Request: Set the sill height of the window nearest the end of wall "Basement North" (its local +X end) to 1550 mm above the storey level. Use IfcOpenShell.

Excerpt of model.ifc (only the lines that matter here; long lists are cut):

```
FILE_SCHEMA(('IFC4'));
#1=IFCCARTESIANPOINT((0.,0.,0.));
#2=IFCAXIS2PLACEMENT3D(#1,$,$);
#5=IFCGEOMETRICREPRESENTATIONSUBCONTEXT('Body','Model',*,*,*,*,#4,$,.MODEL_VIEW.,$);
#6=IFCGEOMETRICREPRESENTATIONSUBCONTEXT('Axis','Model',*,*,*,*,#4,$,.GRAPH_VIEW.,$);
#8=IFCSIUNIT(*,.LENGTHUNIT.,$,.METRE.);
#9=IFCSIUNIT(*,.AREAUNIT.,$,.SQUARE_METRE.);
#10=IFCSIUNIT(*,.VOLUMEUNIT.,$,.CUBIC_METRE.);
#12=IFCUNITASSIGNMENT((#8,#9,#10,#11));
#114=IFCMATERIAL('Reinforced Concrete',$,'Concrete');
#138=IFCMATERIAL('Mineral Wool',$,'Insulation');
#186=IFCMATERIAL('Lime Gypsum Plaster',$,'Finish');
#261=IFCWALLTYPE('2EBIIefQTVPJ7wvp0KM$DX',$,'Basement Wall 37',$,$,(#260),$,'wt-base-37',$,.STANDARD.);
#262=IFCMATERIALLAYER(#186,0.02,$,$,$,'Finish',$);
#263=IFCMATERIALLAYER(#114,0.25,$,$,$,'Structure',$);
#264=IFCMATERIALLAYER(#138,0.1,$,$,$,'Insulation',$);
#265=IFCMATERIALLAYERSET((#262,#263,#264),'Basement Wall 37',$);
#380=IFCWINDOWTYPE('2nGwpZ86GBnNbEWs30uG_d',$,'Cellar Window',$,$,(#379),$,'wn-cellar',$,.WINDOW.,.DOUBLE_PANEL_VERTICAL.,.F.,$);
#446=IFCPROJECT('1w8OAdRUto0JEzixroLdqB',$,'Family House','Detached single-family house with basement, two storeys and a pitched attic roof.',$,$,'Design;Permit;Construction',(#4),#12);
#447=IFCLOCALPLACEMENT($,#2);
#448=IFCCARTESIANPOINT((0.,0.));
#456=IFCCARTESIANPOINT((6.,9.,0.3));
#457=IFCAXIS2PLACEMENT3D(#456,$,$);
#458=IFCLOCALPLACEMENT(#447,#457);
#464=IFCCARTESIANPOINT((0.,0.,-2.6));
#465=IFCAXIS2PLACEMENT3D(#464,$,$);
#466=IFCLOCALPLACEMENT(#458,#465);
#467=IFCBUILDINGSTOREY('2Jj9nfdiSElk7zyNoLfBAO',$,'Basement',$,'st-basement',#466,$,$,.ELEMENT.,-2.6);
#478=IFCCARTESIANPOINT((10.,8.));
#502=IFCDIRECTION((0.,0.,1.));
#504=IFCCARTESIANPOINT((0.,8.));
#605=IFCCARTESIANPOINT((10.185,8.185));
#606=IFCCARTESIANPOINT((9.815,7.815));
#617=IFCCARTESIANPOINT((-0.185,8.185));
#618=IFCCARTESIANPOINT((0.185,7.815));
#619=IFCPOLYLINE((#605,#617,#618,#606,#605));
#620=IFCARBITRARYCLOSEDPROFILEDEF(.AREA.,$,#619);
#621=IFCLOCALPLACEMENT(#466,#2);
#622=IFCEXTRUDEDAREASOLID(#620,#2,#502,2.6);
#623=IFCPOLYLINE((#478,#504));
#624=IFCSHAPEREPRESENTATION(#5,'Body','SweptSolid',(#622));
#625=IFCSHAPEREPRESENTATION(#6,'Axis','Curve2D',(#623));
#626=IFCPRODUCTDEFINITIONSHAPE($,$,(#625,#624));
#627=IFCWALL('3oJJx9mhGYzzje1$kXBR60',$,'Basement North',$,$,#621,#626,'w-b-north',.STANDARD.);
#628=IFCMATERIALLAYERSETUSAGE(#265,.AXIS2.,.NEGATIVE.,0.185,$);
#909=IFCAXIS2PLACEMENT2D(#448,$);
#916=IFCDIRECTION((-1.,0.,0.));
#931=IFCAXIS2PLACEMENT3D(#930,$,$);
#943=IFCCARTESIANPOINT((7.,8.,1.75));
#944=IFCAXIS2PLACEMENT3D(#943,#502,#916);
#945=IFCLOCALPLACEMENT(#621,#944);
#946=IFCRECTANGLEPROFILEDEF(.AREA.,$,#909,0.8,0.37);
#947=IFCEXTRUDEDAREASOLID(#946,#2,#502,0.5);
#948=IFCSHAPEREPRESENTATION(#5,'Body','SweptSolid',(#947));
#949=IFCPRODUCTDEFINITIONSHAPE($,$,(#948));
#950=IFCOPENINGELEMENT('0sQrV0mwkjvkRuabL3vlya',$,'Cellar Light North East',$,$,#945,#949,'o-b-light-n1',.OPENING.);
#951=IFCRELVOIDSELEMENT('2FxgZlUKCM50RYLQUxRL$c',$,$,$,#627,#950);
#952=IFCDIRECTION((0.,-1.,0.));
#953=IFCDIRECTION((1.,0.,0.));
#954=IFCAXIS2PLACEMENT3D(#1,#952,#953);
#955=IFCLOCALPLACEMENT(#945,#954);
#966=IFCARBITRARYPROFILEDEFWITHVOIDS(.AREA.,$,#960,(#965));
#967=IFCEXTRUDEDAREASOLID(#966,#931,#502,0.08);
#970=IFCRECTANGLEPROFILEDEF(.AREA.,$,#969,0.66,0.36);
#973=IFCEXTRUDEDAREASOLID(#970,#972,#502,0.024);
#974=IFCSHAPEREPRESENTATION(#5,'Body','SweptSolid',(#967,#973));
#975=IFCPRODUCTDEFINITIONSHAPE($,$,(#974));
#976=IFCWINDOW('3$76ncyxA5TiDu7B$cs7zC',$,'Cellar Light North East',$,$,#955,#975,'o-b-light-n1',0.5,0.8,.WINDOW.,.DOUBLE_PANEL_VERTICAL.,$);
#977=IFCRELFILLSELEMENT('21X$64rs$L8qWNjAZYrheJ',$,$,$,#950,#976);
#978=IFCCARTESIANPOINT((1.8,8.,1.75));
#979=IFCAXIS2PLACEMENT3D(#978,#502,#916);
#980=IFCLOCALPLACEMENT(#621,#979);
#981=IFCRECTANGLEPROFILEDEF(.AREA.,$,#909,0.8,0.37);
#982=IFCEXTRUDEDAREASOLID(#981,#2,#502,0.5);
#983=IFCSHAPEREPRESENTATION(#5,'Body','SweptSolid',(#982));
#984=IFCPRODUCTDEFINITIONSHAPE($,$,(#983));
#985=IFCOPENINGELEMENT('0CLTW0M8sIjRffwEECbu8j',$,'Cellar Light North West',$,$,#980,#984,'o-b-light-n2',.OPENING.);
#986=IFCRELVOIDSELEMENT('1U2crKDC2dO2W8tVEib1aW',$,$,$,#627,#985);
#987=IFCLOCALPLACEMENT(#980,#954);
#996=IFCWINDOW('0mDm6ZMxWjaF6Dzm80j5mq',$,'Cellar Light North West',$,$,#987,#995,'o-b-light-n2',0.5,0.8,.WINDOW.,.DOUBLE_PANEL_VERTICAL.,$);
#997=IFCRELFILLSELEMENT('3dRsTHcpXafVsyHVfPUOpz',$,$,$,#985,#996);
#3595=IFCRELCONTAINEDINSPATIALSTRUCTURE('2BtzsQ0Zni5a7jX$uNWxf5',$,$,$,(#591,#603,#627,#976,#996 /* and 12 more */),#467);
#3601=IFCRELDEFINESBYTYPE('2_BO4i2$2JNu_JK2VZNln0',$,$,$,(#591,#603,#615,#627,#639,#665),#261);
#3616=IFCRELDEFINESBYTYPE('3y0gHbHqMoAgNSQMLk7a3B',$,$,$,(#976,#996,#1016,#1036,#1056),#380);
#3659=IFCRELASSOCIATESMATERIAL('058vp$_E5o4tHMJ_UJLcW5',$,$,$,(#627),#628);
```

```python
import numpy as np
import ifcopenshell
import ifcopenshell.api.geometry
import ifcopenshell.geom
import ifcopenshell.util.element
import ifcopenshell.util.placement
import ifcopenshell.util.shape
import ifcopenshell.util.unit

model = ifcopenshell.open("model.ifc")
unit_scale = ifcopenshell.util.unit.calculate_unit_scale(model)

window = model.by_guid("3$76ncyxA5TiDu7B$cs7zC")
opening = window.FillsVoids[0].RelatingOpeningElement
storey = ifcopenshell.util.element.get_container(window, ifc_class="IfcBuildingStorey")
level = ifcopenshell.util.placement.get_local_placement(storey.ObjectPlacement)[2, 3]

# The opening's origin need not be at the sill, so measure its lowest point.
shape = ifcopenshell.geom.create_shape(ifcopenshell.geom.settings(), opening)
bottom = ifcopenshell.util.shape.get_shape_bottom_elevation(shape, shape.geometry) / unit_scale
dz = level + 1.55 - bottom

shift = np.array([0.0, 0.0, dz])
# The window is placed relative to its opening, so it follows when the opening moves.
matrix = ifcopenshell.util.placement.get_local_placement(opening.ObjectPlacement)
matrix[:3, 3] += shift
ifcopenshell.api.geometry.edit_object_placement(
    model, product=opening, matrix=matrix, is_si=False, should_transform_children=True
)

print(f"moved by {dz * unit_scale:+.3f} m")

model.write("model_edited.ifc")
```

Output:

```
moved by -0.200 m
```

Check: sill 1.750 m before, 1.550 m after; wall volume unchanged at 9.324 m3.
